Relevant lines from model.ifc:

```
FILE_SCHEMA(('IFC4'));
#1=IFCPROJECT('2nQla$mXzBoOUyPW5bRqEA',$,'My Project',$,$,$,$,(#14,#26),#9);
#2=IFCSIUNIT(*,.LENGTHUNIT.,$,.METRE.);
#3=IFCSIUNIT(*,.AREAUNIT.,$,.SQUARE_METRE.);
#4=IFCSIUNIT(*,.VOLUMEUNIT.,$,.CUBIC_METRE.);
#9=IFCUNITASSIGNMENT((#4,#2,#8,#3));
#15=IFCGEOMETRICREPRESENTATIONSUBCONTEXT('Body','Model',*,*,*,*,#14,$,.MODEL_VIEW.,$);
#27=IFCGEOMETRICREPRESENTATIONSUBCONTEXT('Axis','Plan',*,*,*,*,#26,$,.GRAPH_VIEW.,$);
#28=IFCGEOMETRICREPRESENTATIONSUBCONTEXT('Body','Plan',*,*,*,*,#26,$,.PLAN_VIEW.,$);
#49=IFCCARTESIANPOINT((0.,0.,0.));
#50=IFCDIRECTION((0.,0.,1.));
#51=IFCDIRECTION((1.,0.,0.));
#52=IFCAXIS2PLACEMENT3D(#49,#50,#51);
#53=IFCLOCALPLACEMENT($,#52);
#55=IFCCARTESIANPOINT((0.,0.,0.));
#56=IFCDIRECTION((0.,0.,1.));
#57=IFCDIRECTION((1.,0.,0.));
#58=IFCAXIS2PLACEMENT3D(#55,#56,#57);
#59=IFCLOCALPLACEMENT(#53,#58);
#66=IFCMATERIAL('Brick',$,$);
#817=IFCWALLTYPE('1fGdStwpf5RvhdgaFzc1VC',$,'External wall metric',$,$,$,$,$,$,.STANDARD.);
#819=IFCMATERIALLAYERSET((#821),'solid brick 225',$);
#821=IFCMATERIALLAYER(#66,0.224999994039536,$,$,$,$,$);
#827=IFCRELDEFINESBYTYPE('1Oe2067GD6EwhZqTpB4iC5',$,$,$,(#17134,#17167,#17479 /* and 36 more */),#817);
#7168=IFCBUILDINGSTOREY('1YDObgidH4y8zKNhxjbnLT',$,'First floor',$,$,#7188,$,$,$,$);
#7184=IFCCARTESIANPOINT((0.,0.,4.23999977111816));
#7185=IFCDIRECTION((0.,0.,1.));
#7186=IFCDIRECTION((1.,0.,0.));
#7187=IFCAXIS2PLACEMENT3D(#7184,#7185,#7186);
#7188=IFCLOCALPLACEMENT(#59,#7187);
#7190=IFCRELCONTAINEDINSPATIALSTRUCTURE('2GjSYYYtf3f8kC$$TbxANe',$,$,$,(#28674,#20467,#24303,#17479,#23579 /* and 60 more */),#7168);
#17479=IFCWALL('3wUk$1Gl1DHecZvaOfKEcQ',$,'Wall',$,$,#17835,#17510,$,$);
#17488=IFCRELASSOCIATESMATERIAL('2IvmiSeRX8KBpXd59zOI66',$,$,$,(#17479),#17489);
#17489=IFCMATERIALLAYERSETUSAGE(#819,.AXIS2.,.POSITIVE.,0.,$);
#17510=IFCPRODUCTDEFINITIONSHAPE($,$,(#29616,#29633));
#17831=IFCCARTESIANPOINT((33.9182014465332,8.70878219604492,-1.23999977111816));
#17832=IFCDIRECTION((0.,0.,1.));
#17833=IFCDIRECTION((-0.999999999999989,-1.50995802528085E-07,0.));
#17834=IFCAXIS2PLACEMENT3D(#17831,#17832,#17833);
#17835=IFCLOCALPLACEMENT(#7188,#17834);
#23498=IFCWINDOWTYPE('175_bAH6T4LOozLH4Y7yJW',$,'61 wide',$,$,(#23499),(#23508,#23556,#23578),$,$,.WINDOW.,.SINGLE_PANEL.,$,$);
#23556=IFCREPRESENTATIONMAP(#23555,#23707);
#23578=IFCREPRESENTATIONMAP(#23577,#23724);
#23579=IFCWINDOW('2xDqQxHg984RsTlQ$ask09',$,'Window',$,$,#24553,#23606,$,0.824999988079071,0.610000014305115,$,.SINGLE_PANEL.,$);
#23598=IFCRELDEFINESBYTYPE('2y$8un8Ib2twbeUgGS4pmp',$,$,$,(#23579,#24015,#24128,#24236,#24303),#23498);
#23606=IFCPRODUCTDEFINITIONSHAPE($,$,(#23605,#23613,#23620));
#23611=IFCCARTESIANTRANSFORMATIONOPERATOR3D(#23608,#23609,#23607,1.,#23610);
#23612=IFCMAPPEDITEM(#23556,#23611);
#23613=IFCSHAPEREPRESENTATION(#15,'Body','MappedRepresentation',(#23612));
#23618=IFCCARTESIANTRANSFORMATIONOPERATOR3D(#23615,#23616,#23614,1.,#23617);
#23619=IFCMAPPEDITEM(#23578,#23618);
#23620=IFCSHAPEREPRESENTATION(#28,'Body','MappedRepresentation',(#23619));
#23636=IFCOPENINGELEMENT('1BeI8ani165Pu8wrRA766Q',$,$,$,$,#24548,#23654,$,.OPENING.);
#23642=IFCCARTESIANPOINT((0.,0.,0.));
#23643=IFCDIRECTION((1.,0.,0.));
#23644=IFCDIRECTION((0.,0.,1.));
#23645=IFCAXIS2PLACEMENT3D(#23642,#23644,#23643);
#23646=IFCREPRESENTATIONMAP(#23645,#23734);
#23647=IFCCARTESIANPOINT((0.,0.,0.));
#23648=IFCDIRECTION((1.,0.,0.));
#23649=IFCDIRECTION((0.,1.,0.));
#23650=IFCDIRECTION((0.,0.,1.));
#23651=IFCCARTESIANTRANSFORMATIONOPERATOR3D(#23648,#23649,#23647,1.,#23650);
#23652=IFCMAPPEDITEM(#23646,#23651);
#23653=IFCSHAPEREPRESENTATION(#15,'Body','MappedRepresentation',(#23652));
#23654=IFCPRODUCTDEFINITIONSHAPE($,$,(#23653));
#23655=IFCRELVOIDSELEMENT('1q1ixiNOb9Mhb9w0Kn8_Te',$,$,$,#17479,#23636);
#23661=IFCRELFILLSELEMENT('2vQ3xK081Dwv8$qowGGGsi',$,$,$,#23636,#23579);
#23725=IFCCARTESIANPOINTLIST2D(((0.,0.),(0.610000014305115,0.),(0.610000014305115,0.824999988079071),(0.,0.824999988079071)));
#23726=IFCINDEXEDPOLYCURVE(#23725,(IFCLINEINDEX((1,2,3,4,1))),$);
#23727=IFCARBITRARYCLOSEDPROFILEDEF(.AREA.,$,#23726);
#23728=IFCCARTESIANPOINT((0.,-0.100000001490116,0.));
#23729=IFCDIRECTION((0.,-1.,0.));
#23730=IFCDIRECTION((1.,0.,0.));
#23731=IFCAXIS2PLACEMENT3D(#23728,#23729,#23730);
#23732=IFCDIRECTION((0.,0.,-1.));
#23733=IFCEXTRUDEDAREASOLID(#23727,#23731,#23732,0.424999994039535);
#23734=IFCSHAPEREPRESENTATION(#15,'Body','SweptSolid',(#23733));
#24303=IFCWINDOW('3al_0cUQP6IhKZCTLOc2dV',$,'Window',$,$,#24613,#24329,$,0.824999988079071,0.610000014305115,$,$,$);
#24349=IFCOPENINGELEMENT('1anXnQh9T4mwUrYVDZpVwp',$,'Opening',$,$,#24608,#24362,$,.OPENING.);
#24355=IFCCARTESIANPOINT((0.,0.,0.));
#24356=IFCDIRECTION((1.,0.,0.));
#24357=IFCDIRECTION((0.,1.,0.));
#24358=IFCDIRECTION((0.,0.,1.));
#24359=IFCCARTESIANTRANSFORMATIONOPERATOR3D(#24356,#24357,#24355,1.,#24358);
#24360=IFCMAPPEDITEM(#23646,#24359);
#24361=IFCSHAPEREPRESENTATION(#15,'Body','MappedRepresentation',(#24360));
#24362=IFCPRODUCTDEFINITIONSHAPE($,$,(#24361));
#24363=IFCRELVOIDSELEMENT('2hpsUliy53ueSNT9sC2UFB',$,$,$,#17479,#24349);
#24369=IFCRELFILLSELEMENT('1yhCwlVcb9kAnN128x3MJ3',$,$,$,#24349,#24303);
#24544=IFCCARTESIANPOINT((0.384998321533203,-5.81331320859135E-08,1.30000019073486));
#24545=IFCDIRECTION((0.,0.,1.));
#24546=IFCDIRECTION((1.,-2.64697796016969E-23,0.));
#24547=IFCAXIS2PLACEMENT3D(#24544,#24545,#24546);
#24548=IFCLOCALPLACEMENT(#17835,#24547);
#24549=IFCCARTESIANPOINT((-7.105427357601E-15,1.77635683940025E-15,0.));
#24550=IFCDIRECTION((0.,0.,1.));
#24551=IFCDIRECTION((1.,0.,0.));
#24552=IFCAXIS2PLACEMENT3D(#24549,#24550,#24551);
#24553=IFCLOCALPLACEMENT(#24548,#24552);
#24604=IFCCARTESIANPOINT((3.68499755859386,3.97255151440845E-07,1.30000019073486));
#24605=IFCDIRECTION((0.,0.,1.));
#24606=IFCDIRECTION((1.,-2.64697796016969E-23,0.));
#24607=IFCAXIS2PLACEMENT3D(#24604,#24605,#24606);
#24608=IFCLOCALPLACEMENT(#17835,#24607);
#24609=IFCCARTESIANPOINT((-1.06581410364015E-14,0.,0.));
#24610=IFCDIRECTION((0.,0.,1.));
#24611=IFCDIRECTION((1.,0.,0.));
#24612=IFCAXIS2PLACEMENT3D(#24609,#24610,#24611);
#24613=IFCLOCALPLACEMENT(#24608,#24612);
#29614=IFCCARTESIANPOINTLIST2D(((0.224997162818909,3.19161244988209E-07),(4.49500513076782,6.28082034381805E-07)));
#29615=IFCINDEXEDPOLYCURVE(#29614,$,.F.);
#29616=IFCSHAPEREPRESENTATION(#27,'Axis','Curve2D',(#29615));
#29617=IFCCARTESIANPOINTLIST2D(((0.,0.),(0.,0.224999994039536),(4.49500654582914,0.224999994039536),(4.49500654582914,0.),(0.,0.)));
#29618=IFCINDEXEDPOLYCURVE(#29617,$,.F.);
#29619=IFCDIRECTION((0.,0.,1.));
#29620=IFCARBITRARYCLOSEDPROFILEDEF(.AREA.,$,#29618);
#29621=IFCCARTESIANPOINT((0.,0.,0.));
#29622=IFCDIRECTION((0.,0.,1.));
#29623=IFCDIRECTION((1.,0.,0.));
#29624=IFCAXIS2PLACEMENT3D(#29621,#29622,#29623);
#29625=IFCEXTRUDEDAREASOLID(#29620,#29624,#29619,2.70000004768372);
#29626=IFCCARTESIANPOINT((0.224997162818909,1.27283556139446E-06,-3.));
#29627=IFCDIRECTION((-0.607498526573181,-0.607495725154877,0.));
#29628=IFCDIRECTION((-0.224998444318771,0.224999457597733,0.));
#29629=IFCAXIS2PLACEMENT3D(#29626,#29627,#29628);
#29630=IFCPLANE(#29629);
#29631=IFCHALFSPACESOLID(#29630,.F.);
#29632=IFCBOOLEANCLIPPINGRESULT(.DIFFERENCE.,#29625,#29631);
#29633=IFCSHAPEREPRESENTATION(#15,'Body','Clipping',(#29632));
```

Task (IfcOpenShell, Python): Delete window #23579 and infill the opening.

```python
import ifcopenshell
import ifcopenshell.api.feature
import ifcopenshell.api.root
import ifcopenshell.geom
import ifcopenshell.util.shape

model = ifcopenshell.open("model.ifc")
settings = ifcopenshell.geom.settings()


def volume(element):
    """Net volume in cubic metres, openings subtracted."""
    shape = ifcopenshell.geom.create_shape(settings, element)
    return ifcopenshell.util.shape.get_volume(shape.geometry)


window = model.by_id(23579)
opening = window.FillsVoids[0].RelatingOpeningElement
wall = opening.VoidsElements[0].RelatingBuildingElement
before = volume(wall)

ifcopenshell.api.root.remove_product(model, product=window)
ifcopenshell.api.feature.remove_feature(model, feature=opening)

after = volume(wall)

print(f"wall volume {before:.3f} -> {after:.3f} m3")

model.write("model_rev.ifc")
```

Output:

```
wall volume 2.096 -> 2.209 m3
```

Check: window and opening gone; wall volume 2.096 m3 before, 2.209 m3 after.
